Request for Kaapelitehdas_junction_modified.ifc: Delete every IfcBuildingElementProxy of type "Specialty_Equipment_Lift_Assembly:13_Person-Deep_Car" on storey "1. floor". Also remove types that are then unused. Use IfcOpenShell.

First a look at what the model holds.

```python
import ifcopenshell
import ifcopenshell.util.element

model = ifcopenshell.open("Kaapelitehdas_junction_modified.ifc")
print(model.schema)
storey = next(s for s in model.by_type("IfcBuildingStorey") if s.Name == "1. floor")
proxies = [e for e in ifcopenshell.util.element.get_decomposition(storey) if e.is_a("IfcBuildingElementProxy")]
seen = {}
for e in proxies:
    element_type = ifcopenshell.util.element.get_type(e)
    name = element_type.Name if element_type not in (None, e) else None
    seen[name] = seen.get(name, 0) + 1
for name, count in sorted(seen.items(), key=str):
    print(count, "x", name)
```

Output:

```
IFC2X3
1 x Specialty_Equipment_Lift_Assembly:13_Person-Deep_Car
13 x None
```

```python
import ifcopenshell
import ifcopenshell.api.root
import ifcopenshell.util.element

model = ifcopenshell.open("Kaapelitehdas_junction_modified.ifc")

storey = next(s for s in model.by_type("IfcBuildingStorey") if s.Name == "1. floor")
proxies = [e for e in ifcopenshell.util.element.get_decomposition(storey) if e.is_a("IfcBuildingElementProxy")]
targets = [e for e in proxies if (t := ifcopenshell.util.element.get_type(e)) not in (None, e) and t.Name == "Specialty_Equipment_Lift_Assembly:13_Person-Deep_Car"]
types = {ifcopenshell.util.element.get_type(e) for e in targets} - {None, *targets}

for e in targets:
    ifcopenshell.api.root.remove_product(model, product=e)
print(len(targets), "removed")

unused = [t for t in types if not ifcopenshell.util.element.get_types(t)]
for t in unused:
    ifcopenshell.api.root.remove_product(model, product=t)
print(len(unused), "unused types removed")

model.write("Kaapelitehdas_junction_modified_v2.ifc")
```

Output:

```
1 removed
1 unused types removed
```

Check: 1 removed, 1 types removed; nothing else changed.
